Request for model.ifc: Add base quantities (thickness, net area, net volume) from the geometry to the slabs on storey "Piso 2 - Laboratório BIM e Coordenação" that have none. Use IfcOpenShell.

First a look at what the model holds.

```python
import ifcopenshell
import ifcopenshell.util.element
import ifcopenshell.util.unit

model = ifcopenshell.open("model.ifc")
print(model.schema)
for unit_type in ("LENGTHUNIT", "AREAUNIT", "VOLUMEUNIT"):
    print(unit_type, ifcopenshell.util.unit.calculate_unit_scale(model, unit_type))
storey = next(s for s in model.by_type("IfcBuildingStorey") if s.Name == "Piso 2 - Laboratório BIM e Coordenação")
slabs = [e for e in ifcopenshell.util.element.get_decomposition(storey) if e.is_a("IfcSlab")]
for e in sorted(slabs, key=lambda e: e.id()):
    print(e.id(), e.is_a(), e.Name, list(ifcopenshell.util.element.get_psets(e, qtos_only=True)), sep=" | ")
```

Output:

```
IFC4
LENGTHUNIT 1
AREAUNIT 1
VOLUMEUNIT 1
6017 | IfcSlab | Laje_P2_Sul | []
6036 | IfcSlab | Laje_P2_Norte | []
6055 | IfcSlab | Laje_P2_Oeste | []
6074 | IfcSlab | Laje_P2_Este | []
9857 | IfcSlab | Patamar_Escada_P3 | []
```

```python
import ifcopenshell
import ifcopenshell.api.pset
import ifcopenshell.geom
import ifcopenshell.util.element
import ifcopenshell.util.shape
import ifcopenshell.util.unit

model = ifcopenshell.open("model.ifc")
unit_scale = ifcopenshell.util.unit.calculate_unit_scale(model)
area_scale = ifcopenshell.util.unit.calculate_unit_scale(model, "AREAUNIT")
volume_scale = ifcopenshell.util.unit.calculate_unit_scale(model, "VOLUMEUNIT")
settings = ifcopenshell.geom.settings()

storey = next(s for s in model.by_type("IfcBuildingStorey") if s.Name == "Piso 2 - Laboratório BIM e Coordenação")
slabs = [e for e in ifcopenshell.util.element.get_decomposition(storey) if e.is_a("IfcSlab")]

for e in sorted(slabs, key=lambda e: e.id()):
    if ifcopenshell.util.element.get_psets(e, qtos_only=True, should_inherit=False):
        continue
    # Geometry comes back in metres, in the element's own axes.
    shape = ifcopenshell.geom.create_shape(settings, e)
    values = {
        "Width": ifcopenshell.util.shape.get_z(shape.geometry) / unit_scale,
        "NetArea": ifcopenshell.util.shape.get_footprint_area(shape.geometry) / area_scale,
        "NetVolume": ifcopenshell.util.shape.get_volume(shape.geometry) / volume_scale,
    }
    qto = ifcopenshell.api.pset.add_qto(model, product=e, name="Qto_SlabBaseQuantities")
    ifcopenshell.api.pset.edit_qto(model, qto=qto, properties=values)
    print(e.id(), {k: round(v, 3) for k, v in values.items()})

model.write("model_rev.ifc")
```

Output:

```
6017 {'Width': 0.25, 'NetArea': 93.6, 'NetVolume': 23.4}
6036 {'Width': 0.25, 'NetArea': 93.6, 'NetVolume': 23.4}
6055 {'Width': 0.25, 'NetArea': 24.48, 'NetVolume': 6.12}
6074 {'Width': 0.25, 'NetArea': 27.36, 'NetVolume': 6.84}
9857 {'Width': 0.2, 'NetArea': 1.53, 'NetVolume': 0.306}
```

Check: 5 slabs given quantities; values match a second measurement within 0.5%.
